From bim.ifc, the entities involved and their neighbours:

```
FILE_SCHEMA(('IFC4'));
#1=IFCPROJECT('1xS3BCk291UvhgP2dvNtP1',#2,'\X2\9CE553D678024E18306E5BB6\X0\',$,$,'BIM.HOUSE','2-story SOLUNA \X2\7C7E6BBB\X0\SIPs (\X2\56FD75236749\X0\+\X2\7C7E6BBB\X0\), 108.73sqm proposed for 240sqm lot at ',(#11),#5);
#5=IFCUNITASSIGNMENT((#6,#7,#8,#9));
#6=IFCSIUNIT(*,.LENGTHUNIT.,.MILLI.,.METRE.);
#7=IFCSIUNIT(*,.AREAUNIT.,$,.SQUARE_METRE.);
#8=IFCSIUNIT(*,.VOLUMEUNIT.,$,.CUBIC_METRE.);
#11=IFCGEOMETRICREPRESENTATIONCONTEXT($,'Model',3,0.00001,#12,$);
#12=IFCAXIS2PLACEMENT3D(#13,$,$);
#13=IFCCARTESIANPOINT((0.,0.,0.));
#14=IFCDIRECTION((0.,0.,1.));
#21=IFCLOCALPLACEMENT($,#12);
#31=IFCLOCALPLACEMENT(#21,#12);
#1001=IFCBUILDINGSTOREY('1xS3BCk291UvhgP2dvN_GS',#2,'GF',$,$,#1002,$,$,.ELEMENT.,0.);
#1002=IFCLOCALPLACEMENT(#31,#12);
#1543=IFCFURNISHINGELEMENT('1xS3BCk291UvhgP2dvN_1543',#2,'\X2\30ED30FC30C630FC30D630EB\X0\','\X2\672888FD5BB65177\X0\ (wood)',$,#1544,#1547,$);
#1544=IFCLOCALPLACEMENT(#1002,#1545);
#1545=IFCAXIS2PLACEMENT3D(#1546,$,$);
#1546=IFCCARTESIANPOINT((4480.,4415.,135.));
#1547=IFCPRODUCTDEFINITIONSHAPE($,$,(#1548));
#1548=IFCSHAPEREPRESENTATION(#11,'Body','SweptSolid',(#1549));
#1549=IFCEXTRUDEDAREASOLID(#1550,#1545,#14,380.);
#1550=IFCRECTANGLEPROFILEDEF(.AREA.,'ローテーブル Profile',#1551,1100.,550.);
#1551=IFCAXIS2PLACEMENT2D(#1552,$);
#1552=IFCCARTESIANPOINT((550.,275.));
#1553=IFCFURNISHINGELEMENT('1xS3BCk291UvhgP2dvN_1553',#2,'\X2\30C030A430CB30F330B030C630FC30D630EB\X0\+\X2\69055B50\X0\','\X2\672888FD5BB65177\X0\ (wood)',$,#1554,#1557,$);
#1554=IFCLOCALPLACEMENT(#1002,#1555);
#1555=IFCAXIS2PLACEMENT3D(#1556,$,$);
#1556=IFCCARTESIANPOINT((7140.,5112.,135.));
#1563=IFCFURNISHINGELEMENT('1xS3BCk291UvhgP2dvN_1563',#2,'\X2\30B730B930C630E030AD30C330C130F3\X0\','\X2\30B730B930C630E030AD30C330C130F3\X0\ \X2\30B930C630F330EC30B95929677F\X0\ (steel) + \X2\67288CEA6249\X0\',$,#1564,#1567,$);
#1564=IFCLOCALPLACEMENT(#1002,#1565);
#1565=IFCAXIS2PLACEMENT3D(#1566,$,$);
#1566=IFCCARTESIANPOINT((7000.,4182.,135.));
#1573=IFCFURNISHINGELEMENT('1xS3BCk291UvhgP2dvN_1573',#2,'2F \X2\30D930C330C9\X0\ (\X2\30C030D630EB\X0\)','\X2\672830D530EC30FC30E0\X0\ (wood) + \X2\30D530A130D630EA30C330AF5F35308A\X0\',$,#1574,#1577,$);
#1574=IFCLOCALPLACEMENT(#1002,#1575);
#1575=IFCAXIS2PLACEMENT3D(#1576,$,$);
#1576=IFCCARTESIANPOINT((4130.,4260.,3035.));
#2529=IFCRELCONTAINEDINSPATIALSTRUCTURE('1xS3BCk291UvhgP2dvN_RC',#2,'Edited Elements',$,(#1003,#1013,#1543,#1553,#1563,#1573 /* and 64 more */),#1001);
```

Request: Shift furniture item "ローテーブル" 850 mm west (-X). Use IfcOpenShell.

```python
import ifcopenshell
import ifcopenshell.api.geometry
import ifcopenshell.util.placement

model = ifcopenshell.open("bim.ifc")

item = model.by_guid("1xS3BCk291UvhgP2dvN_1543")
matrix = ifcopenshell.util.placement.get_local_placement(item.ObjectPlacement)
matrix[0, 3] -= 850.0
ifcopenshell.api.geometry.edit_object_placement(model, product=item, matrix=matrix, is_si=False)

print(ifcopenshell.util.placement.get_local_placement(item.ObjectPlacement).round(3) + 0.0)

model.write("bim_v2.ifc")
```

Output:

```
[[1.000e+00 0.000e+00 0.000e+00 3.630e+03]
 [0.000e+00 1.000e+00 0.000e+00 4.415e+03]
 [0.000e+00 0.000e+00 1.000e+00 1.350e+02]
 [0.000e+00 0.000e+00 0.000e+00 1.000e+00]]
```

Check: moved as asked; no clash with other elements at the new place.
